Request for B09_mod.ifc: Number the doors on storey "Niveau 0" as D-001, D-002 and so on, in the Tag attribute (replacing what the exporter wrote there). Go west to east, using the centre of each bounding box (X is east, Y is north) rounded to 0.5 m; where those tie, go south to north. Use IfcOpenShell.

First a look at what the model holds.

```python
import ifcopenshell
import ifcopenshell.util.element
import ifcopenshell.util.placement

model = ifcopenshell.open("B09_mod.ifc")
print(model.schema)
storey = next(s for s in model.by_type("IfcBuildingStorey") if s.Name == "Niveau 0")
doors = [e for e in ifcopenshell.util.element.get_decomposition(storey) if e.is_a("IfcDoor")]
for e in sorted(doors, key=lambda e: e.id()):
    origin = ifcopenshell.util.placement.get_local_placement(e.ObjectPlacement)[:3, 3]
    print(e.id(), e.Tag, e.Name, origin.round(2) + 0.0, sep=" | ")
```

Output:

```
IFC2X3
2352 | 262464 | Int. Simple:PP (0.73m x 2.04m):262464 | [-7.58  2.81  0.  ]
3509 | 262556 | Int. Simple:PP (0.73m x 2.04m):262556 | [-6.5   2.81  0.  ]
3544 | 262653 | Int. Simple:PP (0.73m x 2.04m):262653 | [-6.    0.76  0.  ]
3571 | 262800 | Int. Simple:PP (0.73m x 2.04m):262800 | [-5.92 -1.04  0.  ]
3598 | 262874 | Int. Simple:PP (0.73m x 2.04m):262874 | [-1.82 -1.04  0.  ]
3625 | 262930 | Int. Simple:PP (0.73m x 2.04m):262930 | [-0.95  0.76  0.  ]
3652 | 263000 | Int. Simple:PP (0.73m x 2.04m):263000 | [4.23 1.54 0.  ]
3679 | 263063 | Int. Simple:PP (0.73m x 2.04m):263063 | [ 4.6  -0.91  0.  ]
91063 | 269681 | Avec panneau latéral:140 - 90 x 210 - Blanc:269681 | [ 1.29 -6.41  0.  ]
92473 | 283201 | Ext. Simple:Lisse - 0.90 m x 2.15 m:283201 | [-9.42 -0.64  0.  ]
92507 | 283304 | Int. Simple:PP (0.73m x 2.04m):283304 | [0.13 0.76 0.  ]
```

```python
import ifcopenshell
import ifcopenshell.geom
import ifcopenshell.util.element
import ifcopenshell.util.shape

model = ifcopenshell.open("B09_mod.ifc")
settings = ifcopenshell.geom.settings()
settings.set("use-world-coords", True)


def centre(element):
    shape = ifcopenshell.geom.create_shape(settings, element)
    return ifcopenshell.util.shape.get_bbox_centroid(shape.geometry)


storey = next(s for s in model.by_type("IfcBuildingStorey") if s.Name == "Niveau 0")
doors = [e for e in ifcopenshell.util.element.get_decomposition(storey) if e.is_a("IfcDoor")]

# Insertion points can sit at a corner or the storey origin, so sort by the geometry (in metres).
centres = {e: centre(e) for e in doors}
doors.sort(key=lambda e: (round(centres[e][0] / 0.5), centres[e][1]))

for i, e in enumerate(doors, start=1):
    number = f"D-0{i:02d}"
    e.Tag = number
    print(e.id(), number)

model.write("B09_mod-out.ifc")
```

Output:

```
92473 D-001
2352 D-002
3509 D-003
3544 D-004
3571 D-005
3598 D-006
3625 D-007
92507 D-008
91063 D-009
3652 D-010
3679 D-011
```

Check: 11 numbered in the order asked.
